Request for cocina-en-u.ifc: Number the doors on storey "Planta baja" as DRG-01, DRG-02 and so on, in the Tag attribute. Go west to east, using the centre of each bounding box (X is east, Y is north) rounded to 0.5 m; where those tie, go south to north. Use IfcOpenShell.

First a look at what the model holds.

```python
import ifcopenshell
import ifcopenshell.util.element
import ifcopenshell.util.placement

model = ifcopenshell.open("cocina-en-u.ifc")
print(model.schema)
storey = next(s for s in model.by_type("IfcBuildingStorey") if s.Name == "Planta baja")
doors = [e for e in ifcopenshell.util.element.get_decomposition(storey) if e.is_a("IfcDoor")]
for e in sorted(doors, key=lambda e: e.id()):
    origin = ifcopenshell.util.placement.get_local_placement(e.ObjectPlacement)[:3, 3]
    print(e.id(), e.Tag, e.Name, origin.round(2) + 0.0, sep=" | ")
```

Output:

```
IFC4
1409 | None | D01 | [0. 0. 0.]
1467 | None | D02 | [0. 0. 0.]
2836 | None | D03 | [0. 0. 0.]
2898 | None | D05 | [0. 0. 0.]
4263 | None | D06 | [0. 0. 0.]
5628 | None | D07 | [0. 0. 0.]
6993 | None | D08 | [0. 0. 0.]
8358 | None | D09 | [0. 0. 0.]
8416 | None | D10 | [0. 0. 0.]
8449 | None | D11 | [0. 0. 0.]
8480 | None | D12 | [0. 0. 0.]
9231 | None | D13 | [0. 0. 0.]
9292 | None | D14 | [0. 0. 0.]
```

```python
import ifcopenshell
import ifcopenshell.geom
import ifcopenshell.util.element
import ifcopenshell.util.shape

model = ifcopenshell.open("cocina-en-u.ifc")
settings = ifcopenshell.geom.settings()
settings.set("use-world-coords", True)


def centre(element):
    shape = ifcopenshell.geom.create_shape(settings, element)
    return ifcopenshell.util.shape.get_bbox_centroid(shape.geometry)


storey = next(s for s in model.by_type("IfcBuildingStorey") if s.Name == "Planta baja")
doors = [e for e in ifcopenshell.util.element.get_decomposition(storey) if e.is_a("IfcDoor")]

# Insertion points can sit at a corner or the storey origin, so sort by the geometry (in metres).
centres = {e: centre(e) for e in doors}
doors.sort(key=lambda e: (round(centres[e][0] / 0.5), centres[e][1]))

for i, e in enumerate(doors, start=1):
    number = f"DRG-{i:02d}"
    e.Tag = number
    print(e.id(), number)

model.write("cocina-en-u_updated.ifc")
```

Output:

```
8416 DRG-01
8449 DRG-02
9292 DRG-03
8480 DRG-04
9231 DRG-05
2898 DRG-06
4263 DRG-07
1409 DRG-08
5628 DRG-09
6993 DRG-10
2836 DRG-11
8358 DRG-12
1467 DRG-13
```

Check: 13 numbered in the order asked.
